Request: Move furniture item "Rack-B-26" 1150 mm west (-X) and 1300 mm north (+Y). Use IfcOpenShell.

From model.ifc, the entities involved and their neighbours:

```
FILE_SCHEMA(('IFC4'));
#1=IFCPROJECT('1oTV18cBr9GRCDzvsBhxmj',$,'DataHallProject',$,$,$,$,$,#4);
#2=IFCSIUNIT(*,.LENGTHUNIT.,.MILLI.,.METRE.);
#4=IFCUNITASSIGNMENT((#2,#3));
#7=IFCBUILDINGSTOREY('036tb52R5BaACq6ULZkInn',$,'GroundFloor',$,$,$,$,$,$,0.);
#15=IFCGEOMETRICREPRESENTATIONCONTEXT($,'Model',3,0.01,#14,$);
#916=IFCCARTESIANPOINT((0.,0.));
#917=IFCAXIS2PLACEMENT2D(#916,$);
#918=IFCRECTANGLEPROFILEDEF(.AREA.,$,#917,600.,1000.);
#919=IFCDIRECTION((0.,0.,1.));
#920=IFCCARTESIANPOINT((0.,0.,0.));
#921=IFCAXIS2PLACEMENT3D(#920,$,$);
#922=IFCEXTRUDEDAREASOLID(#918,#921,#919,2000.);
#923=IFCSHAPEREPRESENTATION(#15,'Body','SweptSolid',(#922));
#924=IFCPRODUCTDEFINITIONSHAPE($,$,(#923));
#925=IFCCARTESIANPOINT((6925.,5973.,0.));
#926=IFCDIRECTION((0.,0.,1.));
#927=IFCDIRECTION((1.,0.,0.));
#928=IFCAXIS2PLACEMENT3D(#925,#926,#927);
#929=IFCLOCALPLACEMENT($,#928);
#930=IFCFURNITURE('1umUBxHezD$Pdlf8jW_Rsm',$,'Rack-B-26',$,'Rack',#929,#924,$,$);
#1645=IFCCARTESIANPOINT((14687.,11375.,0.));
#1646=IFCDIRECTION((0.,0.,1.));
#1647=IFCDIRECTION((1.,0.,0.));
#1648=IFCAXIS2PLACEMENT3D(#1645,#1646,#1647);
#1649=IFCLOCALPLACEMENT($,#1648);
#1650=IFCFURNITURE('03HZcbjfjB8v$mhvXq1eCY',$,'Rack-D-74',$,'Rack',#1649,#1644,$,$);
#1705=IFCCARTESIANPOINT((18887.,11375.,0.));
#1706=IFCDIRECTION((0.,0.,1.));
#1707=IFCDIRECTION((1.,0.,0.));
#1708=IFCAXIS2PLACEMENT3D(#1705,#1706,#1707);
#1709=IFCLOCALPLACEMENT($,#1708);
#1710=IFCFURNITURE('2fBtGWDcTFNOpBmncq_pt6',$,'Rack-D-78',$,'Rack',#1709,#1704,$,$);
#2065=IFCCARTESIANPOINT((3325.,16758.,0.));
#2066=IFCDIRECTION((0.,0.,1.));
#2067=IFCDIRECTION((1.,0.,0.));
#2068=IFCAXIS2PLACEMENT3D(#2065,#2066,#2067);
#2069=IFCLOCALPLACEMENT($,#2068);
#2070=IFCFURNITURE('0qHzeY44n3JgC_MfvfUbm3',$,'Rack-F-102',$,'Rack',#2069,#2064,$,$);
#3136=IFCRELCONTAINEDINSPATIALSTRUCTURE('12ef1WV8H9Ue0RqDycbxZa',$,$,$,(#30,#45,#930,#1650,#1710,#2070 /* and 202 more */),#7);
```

```python
import ifcopenshell
import ifcopenshell.api.geometry
import ifcopenshell.util.placement

model = ifcopenshell.open("model.ifc")

item = model.by_guid("1umUBxHezD$Pdlf8jW_Rsm")
matrix = ifcopenshell.util.placement.get_local_placement(item.ObjectPlacement)
matrix[0, 3] -= 1150.0
matrix[1, 3] += 1300.0
ifcopenshell.api.geometry.edit_object_placement(model, product=item, matrix=matrix, is_si=False)

print(ifcopenshell.util.placement.get_local_placement(item.ObjectPlacement).round(3) + 0.0)

model.write("model_edited.ifc")
```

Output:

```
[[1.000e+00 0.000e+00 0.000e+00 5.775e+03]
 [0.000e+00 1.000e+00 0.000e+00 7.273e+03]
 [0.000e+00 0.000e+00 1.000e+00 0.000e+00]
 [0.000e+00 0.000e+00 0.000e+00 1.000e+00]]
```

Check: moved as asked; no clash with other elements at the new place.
